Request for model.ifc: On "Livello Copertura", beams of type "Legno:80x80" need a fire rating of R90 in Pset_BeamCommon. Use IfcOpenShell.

First a look at what the model holds.

```python
import ifcopenshell
import ifcopenshell.util.element

model = ifcopenshell.open("model.ifc")
print(model.schema)
storey = next(s for s in model.by_type("IfcBuildingStorey") if s.Name == "Livello Copertura")
beams = [e for e in ifcopenshell.util.element.get_decomposition(storey) if e.is_a("IfcBeam")]
seen = {}
for e in beams:
    element_type = ifcopenshell.util.element.get_type(e)
    key = (element_type.Name if element_type != e and element_type else None, ifcopenshell.util.element.get_pset(e, "Pset_BeamCommon", "FireRating"))
    seen[key] = seen.get(key, 0) + 1
for (name, value), count in sorted(seen.items(), key=str):
    print(count, "x", name, "|", value)
```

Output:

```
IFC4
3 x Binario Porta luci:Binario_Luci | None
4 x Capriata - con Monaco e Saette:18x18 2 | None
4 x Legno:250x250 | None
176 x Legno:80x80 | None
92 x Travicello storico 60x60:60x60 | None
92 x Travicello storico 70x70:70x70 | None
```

```python
import ifcopenshell
import ifcopenshell.api.pset
import ifcopenshell.util.element

model = ifcopenshell.open("model.ifc")

storey = next(s for s in model.by_type("IfcBuildingStorey") if s.Name == "Livello Copertura")
beams = [e for e in ifcopenshell.util.element.get_decomposition(storey) if e.is_a("IfcBeam")]

count = 0
for e in beams:
    element_type = ifcopenshell.util.element.get_type(e)
    if element_type in (None, e) or element_type.Name != "Legno:80x80":
        continue
    # add_pset returns the element's existing set when there is one.
    pset = ifcopenshell.api.pset.add_pset(model, product=e, name="Pset_BeamCommon")
    ifcopenshell.api.pset.edit_pset(model, pset=pset, properties={"FireRating": "R90"})
    count += 1

print(count, "beams updated")

model.write("model_updated.ifc")
```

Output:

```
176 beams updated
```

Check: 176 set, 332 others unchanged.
